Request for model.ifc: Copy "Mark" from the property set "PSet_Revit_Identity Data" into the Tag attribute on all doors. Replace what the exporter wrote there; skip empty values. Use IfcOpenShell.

First a look at what the model holds.

```python
import ifcopenshell
import ifcopenshell.util.element

model = ifcopenshell.open("model.ifc")
print(model.schema)
doors = model.by_type("IfcDoor")
print(len(doors), "doors")
for e in doors[:8]:
    source = ifcopenshell.util.element.get_pset(e, "PSet_Revit_Identity Data", "Mark")
    target = e.Tag
    print(e.id(), repr(source), repr(target), sep=" | ")
```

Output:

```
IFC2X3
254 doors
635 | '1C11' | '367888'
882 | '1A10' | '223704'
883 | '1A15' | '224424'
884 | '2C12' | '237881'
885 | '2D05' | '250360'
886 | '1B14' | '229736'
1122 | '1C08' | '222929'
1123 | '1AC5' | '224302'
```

```python
import ifcopenshell
import ifcopenshell.util.element

model = ifcopenshell.open("model.ifc")

count = 0
for e in model.by_type("IfcDoor"):
    value = ifcopenshell.util.element.get_pset(e, "PSet_Revit_Identity Data", "Mark")
    current = e.Tag
    if not value or not value.strip() or current == value:
        continue
    e.Tag = value
    count += 1

print(count, "doors updated")

model.write("model_updated.ifc")
```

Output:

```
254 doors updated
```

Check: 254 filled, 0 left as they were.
